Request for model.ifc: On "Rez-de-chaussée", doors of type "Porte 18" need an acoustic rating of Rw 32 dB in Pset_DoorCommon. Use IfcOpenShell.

First a look at what the model holds.

```python
import ifcopenshell
import ifcopenshell.util.element

model = ifcopenshell.open("model.ifc")
print(model.schema)
storey = next(s for s in model.by_type("IfcBuildingStorey") if s.Name == "Rez-de-chaussée")
doors = [e for e in ifcopenshell.util.element.get_decomposition(storey) if e.is_a("IfcDoor")]
seen = {}
for e in doors:
    element_type = ifcopenshell.util.element.get_type(e)
    key = (element_type.Name if element_type != e and element_type else None, ifcopenshell.util.element.get_pset(e, "Pset_DoorCommon", "AcousticRating"))
    seen[key] = seen.get(key, 0) + 1
for (name, value), count in sorted(seen.items(), key=str):
    print(count, "x", name, "|", value)
```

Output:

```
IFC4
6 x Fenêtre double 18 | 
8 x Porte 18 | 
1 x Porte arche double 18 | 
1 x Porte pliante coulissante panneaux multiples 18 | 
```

```python
import ifcopenshell
import ifcopenshell.api.pset
import ifcopenshell.util.element

model = ifcopenshell.open("model.ifc")

storey = next(s for s in model.by_type("IfcBuildingStorey") if s.Name == "Rez-de-chaussée")
doors = [e for e in ifcopenshell.util.element.get_decomposition(storey) if e.is_a("IfcDoor")]

count = 0
for e in doors:
    element_type = ifcopenshell.util.element.get_type(e)
    if element_type in (None, e) or element_type.Name != "Porte 18":
        continue
    # add_pset returns the element's existing set when there is one.
    pset = ifcopenshell.api.pset.add_pset(model, product=e, name="Pset_DoorCommon")
    ifcopenshell.api.pset.edit_pset(model, pset=pset, properties={"AcousticRating": "Rw 32 dB"})
    count += 1

print(count, "doors updated")

model.write("model_edited.ifc")
```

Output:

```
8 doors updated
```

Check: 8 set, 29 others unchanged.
